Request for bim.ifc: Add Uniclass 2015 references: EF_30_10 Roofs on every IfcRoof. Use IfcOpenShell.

First a look at what the model holds.

```python
import ifcopenshell

model = ifcopenshell.open("bim.ifc")
print(model.schema)
print("classifications:", [c.Name for c in model.by_type("IfcClassification")])
for ifc_class in ("IfcDoor", "IfcRoof", "IfcStair", "IfcWall", "IfcWindow"):
    print(ifc_class, len(model.by_type(ifc_class)))
```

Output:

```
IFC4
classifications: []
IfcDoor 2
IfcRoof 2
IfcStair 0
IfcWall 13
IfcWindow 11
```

```python
import ifcopenshell
import ifcopenshell.api.classification

model = ifcopenshell.open("bim.ifc")

system = ifcopenshell.api.classification.add_classification(model, classification="Uniclass 2015")

codes = {
    "IfcRoof": ("EF_30_10", "Roofs"),
}
for ifc_class, (code, name) in codes.items():
    products = model.by_type(ifc_class)
    ifcopenshell.api.classification.add_reference(
        model, products=products, classification=system, identification=code, name=name
    )
    print(code, len(products))

model.write("bim-out.ifc")
```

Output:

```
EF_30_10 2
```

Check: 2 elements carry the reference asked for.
